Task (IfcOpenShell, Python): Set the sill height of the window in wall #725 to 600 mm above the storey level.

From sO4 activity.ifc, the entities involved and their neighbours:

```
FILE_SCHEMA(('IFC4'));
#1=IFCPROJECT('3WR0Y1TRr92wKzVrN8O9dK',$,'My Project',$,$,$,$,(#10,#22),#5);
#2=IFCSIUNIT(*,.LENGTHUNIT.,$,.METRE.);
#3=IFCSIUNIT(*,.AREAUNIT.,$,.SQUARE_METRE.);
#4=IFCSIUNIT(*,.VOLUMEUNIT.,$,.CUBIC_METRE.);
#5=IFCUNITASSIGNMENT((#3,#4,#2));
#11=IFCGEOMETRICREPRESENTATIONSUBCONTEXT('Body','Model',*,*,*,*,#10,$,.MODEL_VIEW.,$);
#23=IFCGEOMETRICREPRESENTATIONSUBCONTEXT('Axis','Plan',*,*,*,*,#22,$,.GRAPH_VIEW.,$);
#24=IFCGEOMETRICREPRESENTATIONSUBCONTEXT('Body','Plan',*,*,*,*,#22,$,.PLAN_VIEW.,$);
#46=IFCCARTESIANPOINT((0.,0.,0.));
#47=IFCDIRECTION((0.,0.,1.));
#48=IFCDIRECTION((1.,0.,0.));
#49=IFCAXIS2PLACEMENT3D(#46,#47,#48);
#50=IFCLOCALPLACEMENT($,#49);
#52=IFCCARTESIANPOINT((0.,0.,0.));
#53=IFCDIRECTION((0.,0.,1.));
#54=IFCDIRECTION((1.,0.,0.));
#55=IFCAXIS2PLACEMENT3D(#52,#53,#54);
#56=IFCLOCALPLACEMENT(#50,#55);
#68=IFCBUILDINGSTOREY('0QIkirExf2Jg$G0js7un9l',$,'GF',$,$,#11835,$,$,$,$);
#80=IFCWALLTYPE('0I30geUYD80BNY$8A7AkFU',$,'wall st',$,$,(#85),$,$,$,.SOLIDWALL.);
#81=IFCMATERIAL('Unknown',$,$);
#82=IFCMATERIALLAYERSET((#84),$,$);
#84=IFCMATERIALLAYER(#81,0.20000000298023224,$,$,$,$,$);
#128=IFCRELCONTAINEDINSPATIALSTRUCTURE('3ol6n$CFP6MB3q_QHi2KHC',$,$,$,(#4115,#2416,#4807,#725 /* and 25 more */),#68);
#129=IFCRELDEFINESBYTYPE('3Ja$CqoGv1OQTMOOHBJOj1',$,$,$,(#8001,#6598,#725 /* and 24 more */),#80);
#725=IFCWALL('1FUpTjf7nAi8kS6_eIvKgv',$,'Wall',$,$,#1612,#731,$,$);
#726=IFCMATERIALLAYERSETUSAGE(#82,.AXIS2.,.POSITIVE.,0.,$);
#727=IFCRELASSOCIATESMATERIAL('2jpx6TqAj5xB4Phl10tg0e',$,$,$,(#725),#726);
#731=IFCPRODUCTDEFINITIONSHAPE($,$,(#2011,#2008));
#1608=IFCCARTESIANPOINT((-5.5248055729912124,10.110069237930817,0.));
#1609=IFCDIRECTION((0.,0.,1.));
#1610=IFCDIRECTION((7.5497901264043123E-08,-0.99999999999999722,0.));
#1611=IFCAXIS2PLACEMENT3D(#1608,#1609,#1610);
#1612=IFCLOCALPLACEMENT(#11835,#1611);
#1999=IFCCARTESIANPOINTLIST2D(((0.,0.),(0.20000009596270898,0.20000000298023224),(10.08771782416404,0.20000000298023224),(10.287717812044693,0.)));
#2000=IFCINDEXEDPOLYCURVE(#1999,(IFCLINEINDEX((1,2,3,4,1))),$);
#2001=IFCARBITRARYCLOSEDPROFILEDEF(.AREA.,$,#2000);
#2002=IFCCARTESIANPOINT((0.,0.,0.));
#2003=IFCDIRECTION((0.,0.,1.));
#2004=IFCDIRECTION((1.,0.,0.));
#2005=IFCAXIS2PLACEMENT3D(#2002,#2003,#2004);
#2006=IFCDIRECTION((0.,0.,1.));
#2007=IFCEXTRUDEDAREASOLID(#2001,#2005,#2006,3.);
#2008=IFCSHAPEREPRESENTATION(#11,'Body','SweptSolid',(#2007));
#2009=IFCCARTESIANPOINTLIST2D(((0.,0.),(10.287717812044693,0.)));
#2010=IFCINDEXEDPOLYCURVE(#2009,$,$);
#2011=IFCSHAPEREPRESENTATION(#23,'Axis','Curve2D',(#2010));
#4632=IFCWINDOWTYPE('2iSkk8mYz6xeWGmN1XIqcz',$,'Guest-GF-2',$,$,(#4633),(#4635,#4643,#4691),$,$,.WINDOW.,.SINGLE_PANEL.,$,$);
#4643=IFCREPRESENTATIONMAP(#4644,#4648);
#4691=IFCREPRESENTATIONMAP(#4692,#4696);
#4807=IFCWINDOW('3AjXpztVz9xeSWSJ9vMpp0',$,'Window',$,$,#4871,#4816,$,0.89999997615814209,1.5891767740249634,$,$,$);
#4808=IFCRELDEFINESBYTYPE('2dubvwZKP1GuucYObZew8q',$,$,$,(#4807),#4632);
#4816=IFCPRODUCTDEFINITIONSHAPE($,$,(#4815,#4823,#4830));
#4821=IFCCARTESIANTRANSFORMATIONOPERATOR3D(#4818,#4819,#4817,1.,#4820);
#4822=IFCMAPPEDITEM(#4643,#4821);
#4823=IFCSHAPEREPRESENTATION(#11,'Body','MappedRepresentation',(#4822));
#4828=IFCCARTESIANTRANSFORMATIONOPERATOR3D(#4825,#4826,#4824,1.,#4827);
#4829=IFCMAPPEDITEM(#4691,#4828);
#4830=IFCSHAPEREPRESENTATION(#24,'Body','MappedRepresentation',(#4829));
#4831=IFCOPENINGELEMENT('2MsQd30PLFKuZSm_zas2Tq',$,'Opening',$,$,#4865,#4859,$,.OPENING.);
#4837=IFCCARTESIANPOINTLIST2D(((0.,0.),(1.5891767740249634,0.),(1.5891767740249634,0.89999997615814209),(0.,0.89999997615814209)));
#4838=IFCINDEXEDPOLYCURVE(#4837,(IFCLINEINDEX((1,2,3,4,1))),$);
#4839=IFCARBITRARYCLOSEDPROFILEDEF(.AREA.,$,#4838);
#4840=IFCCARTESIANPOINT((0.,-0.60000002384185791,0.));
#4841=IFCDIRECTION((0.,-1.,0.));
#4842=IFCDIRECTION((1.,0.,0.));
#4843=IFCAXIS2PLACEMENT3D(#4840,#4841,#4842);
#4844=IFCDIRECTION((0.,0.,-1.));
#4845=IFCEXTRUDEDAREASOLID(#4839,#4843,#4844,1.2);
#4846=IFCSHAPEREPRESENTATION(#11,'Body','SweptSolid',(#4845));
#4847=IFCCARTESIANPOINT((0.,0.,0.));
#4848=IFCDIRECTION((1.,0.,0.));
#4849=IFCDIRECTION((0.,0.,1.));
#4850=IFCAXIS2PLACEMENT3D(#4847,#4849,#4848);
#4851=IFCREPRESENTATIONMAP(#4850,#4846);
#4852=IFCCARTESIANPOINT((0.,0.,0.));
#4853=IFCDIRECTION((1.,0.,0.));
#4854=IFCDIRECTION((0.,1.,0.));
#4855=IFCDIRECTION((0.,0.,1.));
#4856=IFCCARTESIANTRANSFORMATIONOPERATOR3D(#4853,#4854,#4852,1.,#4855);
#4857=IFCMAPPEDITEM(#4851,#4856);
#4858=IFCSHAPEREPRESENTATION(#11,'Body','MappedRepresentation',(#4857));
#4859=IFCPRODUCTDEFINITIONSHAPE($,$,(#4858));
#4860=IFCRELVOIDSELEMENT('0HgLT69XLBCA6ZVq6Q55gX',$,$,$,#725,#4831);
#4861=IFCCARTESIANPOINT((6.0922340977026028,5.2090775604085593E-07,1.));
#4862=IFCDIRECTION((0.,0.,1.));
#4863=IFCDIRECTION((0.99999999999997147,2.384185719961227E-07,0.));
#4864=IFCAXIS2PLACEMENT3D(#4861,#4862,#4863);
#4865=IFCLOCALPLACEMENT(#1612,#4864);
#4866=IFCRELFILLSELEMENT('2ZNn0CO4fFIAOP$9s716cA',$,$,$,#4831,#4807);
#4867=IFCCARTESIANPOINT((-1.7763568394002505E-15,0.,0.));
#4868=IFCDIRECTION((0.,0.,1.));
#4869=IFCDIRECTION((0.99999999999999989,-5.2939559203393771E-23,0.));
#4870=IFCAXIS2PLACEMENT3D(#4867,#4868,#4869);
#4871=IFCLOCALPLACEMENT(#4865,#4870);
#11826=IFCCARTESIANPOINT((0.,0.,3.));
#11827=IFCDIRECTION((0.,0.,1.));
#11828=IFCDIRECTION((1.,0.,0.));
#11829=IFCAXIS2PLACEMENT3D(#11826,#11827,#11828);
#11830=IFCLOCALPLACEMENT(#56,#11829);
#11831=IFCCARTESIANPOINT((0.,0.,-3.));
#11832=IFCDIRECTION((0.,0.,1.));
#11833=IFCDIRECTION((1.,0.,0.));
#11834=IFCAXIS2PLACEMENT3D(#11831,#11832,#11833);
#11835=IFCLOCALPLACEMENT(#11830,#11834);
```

```python
import numpy as np
import ifcopenshell
import ifcopenshell.api.geometry
import ifcopenshell.geom
import ifcopenshell.util.element
import ifcopenshell.util.placement
import ifcopenshell.util.shape
import ifcopenshell.util.unit

model = ifcopenshell.open("sO4 activity.ifc")
unit_scale = ifcopenshell.util.unit.calculate_unit_scale(model)

window = model.by_guid("3AjXpztVz9xeSWSJ9vMpp0")
opening = window.FillsVoids[0].RelatingOpeningElement
storey = ifcopenshell.util.element.get_container(window, ifc_class="IfcBuildingStorey")
level = ifcopenshell.util.placement.get_local_placement(storey.ObjectPlacement)[2, 3]

# The opening's origin need not be at the sill, so measure its lowest point.
shape = ifcopenshell.geom.create_shape(ifcopenshell.geom.settings(), opening)
bottom = ifcopenshell.util.shape.get_shape_bottom_elevation(shape, shape.geometry) / unit_scale
dz = level + 0.6 / unit_scale - bottom

shift = np.array([0.0, 0.0, dz])
# The window is placed relative to its opening, so it follows when the opening moves.
matrix = ifcopenshell.util.placement.get_local_placement(opening.ObjectPlacement)
matrix[:3, 3] += shift
ifcopenshell.api.geometry.edit_object_placement(
    model, product=opening, matrix=matrix, is_si=False, should_transform_children=True
)

print(f"moved by {dz * unit_scale:+.3f} m")

model.write("sO4 activity_rev.ifc")
```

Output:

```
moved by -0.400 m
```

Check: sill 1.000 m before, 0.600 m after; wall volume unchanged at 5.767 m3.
